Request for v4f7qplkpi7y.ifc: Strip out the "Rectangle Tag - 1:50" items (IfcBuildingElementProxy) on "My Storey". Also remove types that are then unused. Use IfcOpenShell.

First a look at what the model holds.

```python
import ifcopenshell
import ifcopenshell.util.element

model = ifcopenshell.open("v4f7qplkpi7y.ifc")
print(model.schema)
storey = next(s for s in model.by_type("IfcBuildingStorey") if s.Name == "My Storey")
proxies = [e for e in ifcopenshell.util.element.get_decomposition(storey) if e.is_a("IfcBuildingElementProxy")]
seen = {}
for e in proxies:
    element_type = ifcopenshell.util.element.get_type(e)
    name = element_type.Name if element_type not in (None, e) else None
    seen[name] = seen.get(name, 0) + 1
for name, count in sorted(seen.items(), key=str):
    print(count, "x", name)
```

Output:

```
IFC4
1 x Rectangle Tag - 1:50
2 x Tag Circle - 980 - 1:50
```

```python
import ifcopenshell
import ifcopenshell.api.root
import ifcopenshell.util.element

model = ifcopenshell.open("v4f7qplkpi7y.ifc")

storey = next(s for s in model.by_type("IfcBuildingStorey") if s.Name == "My Storey")
proxies = [e for e in ifcopenshell.util.element.get_decomposition(storey) if e.is_a("IfcBuildingElementProxy")]
targets = [e for e in proxies if (t := ifcopenshell.util.element.get_type(e)) not in (None, e) and t.Name == "Rectangle Tag - 1:50"]
types = {ifcopenshell.util.element.get_type(e) for e in targets} - {None, *targets}

for e in targets:
    ifcopenshell.api.root.remove_product(model, product=e)
print(len(targets), "removed")

unused = [t for t in types if not ifcopenshell.util.element.get_types(t)]
for t in unused:
    ifcopenshell.api.root.remove_product(model, product=t)
print(len(unused), "unused types removed")

model.write("v4f7qplkpi7y_v2.ifc")
```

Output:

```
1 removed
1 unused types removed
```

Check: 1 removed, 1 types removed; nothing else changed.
